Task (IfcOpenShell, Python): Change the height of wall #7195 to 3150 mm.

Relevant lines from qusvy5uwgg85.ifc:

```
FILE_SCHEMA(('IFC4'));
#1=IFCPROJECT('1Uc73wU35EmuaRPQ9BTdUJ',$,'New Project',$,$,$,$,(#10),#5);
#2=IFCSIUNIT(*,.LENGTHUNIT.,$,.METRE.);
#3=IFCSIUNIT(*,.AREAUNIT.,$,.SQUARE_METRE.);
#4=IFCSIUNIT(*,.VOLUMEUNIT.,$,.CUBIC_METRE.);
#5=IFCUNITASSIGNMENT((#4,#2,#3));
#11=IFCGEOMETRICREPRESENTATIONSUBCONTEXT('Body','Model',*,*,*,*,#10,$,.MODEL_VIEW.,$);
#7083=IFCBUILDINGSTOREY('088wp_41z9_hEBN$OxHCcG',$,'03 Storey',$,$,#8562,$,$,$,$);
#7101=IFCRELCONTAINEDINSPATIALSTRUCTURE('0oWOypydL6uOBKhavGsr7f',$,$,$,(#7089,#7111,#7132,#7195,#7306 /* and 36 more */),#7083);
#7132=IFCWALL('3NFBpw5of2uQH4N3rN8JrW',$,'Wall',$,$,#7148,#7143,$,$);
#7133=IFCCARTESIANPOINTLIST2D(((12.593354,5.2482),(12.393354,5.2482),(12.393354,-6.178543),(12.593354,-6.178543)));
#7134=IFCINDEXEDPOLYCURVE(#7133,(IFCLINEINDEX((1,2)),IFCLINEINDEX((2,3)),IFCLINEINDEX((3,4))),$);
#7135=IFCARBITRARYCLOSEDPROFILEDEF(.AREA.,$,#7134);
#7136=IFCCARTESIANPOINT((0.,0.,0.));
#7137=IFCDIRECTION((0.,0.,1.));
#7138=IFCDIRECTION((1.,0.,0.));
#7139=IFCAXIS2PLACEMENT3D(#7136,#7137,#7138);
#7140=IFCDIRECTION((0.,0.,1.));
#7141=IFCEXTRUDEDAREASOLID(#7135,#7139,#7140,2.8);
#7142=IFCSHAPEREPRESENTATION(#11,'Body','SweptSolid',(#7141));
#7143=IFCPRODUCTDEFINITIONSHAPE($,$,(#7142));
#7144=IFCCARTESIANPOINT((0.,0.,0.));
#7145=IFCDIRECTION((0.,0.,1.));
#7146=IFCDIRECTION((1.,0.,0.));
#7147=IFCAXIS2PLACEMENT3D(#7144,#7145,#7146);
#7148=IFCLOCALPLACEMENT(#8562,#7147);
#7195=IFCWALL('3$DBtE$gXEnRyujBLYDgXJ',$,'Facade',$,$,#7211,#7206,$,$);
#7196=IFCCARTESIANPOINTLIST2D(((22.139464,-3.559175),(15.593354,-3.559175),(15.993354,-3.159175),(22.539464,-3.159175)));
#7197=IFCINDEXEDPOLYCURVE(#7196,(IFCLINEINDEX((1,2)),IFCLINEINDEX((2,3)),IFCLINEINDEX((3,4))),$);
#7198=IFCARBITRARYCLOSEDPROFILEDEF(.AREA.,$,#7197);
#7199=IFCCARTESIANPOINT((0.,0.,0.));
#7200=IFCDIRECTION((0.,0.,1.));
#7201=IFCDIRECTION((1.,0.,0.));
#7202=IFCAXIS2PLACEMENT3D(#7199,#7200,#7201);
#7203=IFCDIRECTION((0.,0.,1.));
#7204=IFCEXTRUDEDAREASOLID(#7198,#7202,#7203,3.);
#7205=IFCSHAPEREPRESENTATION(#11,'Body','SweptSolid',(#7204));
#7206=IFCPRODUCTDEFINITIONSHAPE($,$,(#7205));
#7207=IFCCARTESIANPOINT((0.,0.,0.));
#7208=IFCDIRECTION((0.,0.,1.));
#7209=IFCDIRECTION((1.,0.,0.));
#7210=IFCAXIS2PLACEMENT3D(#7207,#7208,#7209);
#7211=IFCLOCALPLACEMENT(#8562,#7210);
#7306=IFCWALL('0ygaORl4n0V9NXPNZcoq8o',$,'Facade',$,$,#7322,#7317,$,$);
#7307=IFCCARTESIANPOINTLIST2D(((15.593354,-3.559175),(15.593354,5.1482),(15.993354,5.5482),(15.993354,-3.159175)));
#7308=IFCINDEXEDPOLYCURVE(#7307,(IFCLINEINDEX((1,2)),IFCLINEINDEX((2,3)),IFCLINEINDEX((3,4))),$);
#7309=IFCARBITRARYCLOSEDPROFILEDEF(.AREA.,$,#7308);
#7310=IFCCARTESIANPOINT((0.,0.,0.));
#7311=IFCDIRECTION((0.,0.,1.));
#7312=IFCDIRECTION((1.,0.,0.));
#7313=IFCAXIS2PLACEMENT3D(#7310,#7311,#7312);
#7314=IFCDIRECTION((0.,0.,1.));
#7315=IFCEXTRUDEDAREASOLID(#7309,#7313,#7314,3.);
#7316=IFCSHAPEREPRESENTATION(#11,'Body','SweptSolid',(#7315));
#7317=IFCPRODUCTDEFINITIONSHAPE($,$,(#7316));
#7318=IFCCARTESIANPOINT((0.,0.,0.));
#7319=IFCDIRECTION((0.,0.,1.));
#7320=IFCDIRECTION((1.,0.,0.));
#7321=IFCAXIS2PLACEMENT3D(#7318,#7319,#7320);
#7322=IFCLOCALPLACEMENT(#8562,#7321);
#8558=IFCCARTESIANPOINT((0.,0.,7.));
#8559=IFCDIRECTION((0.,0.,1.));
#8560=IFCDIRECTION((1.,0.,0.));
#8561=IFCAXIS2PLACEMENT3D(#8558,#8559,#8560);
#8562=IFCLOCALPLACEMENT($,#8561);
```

```python
import ifcopenshell
import ifcopenshell.geom
import ifcopenshell.util.representation
import ifcopenshell.util.shape
import ifcopenshell.util.unit

model = ifcopenshell.open("qusvy5uwgg85.ifc")
unit_scale = ifcopenshell.util.unit.calculate_unit_scale(model)
settings = ifcopenshell.geom.settings()


def volume(element):
    """Net volume in cubic metres, openings subtracted."""
    shape = ifcopenshell.geom.create_shape(settings, element)
    return ifcopenshell.util.shape.get_volume(shape.geometry)


wall = model.by_id(7195)
before = volume(wall)

body = ifcopenshell.util.representation.get_representation(wall, "Model", "Body")
solid = body.Items[0]
old_height = solid.Depth
solid.Depth = 3.15 / unit_scale
after = volume(wall)

print(f"height {old_height:g} -> {solid.Depth:g}, volume {before:.3f} -> {after:.3f} m3")

model.write("qusvy5uwgg85-out.ifc")
```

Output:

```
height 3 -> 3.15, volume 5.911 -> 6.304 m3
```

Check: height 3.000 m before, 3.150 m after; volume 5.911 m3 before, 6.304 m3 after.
